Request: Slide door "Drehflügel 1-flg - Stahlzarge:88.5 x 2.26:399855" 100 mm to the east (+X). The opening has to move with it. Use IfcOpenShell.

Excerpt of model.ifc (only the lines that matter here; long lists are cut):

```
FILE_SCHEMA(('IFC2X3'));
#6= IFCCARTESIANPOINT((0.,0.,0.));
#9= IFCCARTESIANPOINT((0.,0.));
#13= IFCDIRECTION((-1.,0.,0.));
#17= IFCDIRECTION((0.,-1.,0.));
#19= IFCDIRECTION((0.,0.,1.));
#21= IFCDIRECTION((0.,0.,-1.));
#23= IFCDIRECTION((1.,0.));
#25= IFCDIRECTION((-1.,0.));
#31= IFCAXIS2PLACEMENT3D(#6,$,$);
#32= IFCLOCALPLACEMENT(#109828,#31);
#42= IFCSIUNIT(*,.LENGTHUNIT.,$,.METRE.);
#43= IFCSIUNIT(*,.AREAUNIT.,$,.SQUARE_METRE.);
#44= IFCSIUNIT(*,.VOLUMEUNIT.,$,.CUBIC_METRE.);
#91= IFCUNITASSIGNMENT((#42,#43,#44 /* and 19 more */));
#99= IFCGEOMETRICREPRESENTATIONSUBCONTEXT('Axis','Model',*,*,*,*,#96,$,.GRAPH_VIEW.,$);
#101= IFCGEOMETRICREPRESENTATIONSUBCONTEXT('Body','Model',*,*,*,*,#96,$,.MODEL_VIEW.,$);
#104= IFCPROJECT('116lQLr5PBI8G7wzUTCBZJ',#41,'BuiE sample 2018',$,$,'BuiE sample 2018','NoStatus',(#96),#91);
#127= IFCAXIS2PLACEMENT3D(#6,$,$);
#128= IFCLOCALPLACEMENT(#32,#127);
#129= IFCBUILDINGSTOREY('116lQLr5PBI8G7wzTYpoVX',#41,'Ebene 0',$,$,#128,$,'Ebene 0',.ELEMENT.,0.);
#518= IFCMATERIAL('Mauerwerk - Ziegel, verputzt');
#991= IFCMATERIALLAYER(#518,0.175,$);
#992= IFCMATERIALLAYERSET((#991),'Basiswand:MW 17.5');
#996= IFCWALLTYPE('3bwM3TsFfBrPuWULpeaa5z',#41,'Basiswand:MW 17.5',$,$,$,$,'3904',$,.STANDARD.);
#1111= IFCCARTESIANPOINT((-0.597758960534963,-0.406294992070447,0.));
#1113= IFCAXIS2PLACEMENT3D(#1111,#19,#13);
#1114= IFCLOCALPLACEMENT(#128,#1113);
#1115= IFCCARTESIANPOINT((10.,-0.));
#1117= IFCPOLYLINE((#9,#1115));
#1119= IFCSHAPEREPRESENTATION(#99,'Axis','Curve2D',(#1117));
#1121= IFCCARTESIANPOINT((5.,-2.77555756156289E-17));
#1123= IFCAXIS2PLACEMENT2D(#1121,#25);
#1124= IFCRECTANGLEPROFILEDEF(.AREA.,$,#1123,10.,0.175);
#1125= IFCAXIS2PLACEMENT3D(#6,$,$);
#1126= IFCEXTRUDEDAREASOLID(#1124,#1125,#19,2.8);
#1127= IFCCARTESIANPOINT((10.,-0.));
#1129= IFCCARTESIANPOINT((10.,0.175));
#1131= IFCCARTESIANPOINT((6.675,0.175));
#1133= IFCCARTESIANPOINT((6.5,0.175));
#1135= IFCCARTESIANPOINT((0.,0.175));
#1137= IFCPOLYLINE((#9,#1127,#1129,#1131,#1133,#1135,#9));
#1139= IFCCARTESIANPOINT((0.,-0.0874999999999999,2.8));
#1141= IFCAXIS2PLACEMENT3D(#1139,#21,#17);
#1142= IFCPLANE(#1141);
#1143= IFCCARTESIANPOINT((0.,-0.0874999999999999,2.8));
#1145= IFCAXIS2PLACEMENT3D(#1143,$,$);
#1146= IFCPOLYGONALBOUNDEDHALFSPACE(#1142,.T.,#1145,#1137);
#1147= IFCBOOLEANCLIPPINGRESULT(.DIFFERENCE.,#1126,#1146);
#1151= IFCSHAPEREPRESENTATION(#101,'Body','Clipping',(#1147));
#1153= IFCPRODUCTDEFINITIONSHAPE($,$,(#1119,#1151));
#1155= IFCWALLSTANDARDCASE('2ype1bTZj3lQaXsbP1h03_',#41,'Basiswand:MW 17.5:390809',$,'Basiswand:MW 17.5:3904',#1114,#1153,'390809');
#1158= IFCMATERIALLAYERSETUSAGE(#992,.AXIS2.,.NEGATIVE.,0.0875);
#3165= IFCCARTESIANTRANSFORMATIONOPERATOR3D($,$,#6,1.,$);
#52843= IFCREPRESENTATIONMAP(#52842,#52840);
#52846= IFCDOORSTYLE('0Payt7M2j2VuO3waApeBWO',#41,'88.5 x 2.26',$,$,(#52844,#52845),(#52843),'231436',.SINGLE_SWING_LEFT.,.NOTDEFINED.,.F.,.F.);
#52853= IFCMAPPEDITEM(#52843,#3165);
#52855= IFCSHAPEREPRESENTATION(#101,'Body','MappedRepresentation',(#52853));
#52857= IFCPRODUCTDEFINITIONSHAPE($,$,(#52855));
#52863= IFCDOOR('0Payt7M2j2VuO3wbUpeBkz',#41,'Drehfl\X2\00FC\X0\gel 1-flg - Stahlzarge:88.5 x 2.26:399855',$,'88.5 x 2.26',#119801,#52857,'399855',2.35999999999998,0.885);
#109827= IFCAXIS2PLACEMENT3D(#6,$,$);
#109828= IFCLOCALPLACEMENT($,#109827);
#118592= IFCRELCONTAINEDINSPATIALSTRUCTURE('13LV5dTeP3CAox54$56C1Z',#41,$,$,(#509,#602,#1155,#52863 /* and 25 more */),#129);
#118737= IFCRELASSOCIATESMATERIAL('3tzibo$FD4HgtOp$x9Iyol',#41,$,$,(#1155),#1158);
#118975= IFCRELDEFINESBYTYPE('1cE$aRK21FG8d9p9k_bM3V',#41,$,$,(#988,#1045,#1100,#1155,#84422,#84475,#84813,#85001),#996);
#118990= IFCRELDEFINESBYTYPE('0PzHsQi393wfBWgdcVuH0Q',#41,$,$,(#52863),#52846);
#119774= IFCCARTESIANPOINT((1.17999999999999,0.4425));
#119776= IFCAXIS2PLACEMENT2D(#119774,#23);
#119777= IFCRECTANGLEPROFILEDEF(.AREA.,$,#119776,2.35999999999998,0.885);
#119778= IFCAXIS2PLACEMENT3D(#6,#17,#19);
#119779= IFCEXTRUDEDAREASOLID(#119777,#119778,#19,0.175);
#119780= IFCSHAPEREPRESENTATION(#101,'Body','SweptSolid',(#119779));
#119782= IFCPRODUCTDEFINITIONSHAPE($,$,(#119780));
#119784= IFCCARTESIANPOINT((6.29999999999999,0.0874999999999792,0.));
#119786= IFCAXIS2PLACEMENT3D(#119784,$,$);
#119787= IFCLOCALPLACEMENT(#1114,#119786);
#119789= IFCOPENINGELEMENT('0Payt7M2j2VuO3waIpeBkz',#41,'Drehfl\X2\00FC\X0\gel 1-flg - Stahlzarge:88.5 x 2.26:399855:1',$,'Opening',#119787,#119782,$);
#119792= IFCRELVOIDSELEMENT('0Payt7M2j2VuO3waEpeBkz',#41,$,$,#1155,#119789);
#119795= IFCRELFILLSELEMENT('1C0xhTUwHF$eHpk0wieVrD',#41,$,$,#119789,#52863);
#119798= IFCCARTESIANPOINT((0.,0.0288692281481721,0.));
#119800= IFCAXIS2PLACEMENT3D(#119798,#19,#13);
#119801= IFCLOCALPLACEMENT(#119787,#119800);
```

```python
import ifcopenshell
import ifcopenshell.api.geometry
import ifcopenshell.util.placement

model = ifcopenshell.open("model.ifc")

door = model.by_id(52863)
opening = door.FillsVoids[0].RelatingOpeningElement
wall = opening.VoidsElements[0].RelatingBuildingElement

wall_matrix = ifcopenshell.util.placement.get_local_placement(wall.ObjectPlacement)
shift = wall_matrix[:3, 0] * -0.1
before = ifcopenshell.util.placement.get_local_placement(door.ObjectPlacement)[:3, 3].copy()

# The door is placed relative to its opening, so it follows when the opening moves.
matrix = ifcopenshell.util.placement.get_local_placement(opening.ObjectPlacement)
matrix[:3, 3] += shift
ifcopenshell.api.geometry.edit_object_placement(
    model, product=opening, matrix=matrix, is_si=False, should_transform_children=True
)

after = ifcopenshell.util.placement.get_local_placement(door.ObjectPlacement)[:3, 3]
print("door moved by", (after - before).round(3) + 0.0)

model.write("model_edited.ifc")
```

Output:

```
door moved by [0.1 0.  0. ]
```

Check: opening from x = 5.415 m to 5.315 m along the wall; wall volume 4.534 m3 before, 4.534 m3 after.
